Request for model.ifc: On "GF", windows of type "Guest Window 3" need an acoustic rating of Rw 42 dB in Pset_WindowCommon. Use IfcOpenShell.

First a look at what the model holds.

```python
import ifcopenshell
import ifcopenshell.util.element

model = ifcopenshell.open("model.ifc")
print(model.schema)
storey = next(s for s in model.by_type("IfcBuildingStorey") if s.Name == "GF")
windows = [e for e in ifcopenshell.util.element.get_decomposition(storey) if e.is_a("IfcWindow")]
seen = {}
for e in windows:
    element_type = ifcopenshell.util.element.get_type(e)
    key = (element_type.Name if element_type != e and element_type else None, ifcopenshell.util.element.get_pset(e, "Pset_WindowCommon", "AcousticRating"))
    seen[key] = seen.get(key, 0) + 1
for (name, value), count in sorted(seen.items(), key=str):
    print(count, "x", name, "|", value)
```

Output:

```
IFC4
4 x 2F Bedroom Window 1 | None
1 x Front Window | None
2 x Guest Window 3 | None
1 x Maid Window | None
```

```python
import ifcopenshell
import ifcopenshell.api.pset
import ifcopenshell.util.element

model = ifcopenshell.open("model.ifc")

storey = next(s for s in model.by_type("IfcBuildingStorey") if s.Name == "GF")
windows = [e for e in ifcopenshell.util.element.get_decomposition(storey) if e.is_a("IfcWindow")]

count = 0
for e in windows:
    element_type = ifcopenshell.util.element.get_type(e)
    if element_type in (None, e) or element_type.Name != "Guest Window 3":
        continue
    # add_pset returns the element's existing set when there is one.
    pset = ifcopenshell.api.pset.add_pset(model, product=e, name="Pset_WindowCommon")
    ifcopenshell.api.pset.edit_pset(model, pset=pset, properties={"AcousticRating": "Rw 42 dB"})
    count += 1

print(count, "windows updated")

model.write("model_updated.ifc")
```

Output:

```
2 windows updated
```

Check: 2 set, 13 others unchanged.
